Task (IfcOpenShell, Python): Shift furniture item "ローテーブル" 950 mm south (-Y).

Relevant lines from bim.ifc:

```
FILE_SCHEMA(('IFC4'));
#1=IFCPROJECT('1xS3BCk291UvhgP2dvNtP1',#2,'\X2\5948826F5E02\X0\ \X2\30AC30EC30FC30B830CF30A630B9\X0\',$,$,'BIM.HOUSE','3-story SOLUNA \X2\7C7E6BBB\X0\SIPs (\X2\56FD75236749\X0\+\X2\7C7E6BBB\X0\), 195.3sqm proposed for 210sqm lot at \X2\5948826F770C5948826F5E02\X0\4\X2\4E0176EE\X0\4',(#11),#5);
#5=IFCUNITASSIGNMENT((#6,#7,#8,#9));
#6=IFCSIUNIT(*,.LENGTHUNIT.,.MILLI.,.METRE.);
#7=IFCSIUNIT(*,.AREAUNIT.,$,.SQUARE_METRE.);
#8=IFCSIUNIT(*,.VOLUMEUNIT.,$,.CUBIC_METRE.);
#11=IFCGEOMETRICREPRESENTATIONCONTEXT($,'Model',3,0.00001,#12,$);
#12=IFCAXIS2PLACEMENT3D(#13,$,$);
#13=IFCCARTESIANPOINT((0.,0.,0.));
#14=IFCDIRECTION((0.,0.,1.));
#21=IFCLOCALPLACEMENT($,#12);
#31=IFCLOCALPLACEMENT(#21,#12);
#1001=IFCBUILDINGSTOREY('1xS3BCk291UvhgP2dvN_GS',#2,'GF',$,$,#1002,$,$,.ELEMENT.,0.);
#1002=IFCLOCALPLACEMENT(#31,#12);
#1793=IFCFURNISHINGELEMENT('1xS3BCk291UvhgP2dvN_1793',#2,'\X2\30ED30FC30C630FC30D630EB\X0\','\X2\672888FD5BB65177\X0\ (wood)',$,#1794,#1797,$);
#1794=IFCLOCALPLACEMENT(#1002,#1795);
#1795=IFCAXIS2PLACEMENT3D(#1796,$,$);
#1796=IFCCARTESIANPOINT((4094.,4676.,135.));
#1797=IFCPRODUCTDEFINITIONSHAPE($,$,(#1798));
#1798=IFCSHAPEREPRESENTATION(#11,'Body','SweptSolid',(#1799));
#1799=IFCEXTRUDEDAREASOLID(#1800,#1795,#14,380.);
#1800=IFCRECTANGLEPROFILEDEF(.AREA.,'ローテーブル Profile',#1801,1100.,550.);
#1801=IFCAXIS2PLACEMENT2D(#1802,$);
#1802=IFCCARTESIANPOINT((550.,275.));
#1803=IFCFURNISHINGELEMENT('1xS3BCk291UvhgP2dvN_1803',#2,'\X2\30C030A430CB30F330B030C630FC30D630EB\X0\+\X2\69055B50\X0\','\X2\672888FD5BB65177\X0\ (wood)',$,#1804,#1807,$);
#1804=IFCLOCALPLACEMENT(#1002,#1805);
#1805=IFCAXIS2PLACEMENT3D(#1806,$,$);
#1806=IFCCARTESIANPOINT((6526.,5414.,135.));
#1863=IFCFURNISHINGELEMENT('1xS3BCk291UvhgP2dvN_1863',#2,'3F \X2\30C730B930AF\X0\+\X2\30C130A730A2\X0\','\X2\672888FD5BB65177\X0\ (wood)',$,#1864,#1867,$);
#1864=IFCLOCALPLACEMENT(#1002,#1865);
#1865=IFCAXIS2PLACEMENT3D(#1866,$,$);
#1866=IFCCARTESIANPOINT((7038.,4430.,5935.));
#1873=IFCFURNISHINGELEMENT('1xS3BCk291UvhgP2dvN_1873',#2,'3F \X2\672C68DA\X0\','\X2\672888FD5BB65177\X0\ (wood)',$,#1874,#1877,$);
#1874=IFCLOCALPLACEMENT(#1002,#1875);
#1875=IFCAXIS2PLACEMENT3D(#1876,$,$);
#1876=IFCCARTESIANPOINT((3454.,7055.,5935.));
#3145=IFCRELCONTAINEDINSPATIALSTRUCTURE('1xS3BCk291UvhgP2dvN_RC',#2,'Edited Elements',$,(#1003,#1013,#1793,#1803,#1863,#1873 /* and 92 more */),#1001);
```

```python
import ifcopenshell
import ifcopenshell.api.geometry
import ifcopenshell.util.placement

model = ifcopenshell.open("bim.ifc")

item = model.by_id(1793)
matrix = ifcopenshell.util.placement.get_local_placement(item.ObjectPlacement)
matrix[1, 3] -= 950.0
ifcopenshell.api.geometry.edit_object_placement(model, product=item, matrix=matrix, is_si=False)

print(ifcopenshell.util.placement.get_local_placement(item.ObjectPlacement).round(3) + 0.0)

model.write("bim_edited.ifc")
```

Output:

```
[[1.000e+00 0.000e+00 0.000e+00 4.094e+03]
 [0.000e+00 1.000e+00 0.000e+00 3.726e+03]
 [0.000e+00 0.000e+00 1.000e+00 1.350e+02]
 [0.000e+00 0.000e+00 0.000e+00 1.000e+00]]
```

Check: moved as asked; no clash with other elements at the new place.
